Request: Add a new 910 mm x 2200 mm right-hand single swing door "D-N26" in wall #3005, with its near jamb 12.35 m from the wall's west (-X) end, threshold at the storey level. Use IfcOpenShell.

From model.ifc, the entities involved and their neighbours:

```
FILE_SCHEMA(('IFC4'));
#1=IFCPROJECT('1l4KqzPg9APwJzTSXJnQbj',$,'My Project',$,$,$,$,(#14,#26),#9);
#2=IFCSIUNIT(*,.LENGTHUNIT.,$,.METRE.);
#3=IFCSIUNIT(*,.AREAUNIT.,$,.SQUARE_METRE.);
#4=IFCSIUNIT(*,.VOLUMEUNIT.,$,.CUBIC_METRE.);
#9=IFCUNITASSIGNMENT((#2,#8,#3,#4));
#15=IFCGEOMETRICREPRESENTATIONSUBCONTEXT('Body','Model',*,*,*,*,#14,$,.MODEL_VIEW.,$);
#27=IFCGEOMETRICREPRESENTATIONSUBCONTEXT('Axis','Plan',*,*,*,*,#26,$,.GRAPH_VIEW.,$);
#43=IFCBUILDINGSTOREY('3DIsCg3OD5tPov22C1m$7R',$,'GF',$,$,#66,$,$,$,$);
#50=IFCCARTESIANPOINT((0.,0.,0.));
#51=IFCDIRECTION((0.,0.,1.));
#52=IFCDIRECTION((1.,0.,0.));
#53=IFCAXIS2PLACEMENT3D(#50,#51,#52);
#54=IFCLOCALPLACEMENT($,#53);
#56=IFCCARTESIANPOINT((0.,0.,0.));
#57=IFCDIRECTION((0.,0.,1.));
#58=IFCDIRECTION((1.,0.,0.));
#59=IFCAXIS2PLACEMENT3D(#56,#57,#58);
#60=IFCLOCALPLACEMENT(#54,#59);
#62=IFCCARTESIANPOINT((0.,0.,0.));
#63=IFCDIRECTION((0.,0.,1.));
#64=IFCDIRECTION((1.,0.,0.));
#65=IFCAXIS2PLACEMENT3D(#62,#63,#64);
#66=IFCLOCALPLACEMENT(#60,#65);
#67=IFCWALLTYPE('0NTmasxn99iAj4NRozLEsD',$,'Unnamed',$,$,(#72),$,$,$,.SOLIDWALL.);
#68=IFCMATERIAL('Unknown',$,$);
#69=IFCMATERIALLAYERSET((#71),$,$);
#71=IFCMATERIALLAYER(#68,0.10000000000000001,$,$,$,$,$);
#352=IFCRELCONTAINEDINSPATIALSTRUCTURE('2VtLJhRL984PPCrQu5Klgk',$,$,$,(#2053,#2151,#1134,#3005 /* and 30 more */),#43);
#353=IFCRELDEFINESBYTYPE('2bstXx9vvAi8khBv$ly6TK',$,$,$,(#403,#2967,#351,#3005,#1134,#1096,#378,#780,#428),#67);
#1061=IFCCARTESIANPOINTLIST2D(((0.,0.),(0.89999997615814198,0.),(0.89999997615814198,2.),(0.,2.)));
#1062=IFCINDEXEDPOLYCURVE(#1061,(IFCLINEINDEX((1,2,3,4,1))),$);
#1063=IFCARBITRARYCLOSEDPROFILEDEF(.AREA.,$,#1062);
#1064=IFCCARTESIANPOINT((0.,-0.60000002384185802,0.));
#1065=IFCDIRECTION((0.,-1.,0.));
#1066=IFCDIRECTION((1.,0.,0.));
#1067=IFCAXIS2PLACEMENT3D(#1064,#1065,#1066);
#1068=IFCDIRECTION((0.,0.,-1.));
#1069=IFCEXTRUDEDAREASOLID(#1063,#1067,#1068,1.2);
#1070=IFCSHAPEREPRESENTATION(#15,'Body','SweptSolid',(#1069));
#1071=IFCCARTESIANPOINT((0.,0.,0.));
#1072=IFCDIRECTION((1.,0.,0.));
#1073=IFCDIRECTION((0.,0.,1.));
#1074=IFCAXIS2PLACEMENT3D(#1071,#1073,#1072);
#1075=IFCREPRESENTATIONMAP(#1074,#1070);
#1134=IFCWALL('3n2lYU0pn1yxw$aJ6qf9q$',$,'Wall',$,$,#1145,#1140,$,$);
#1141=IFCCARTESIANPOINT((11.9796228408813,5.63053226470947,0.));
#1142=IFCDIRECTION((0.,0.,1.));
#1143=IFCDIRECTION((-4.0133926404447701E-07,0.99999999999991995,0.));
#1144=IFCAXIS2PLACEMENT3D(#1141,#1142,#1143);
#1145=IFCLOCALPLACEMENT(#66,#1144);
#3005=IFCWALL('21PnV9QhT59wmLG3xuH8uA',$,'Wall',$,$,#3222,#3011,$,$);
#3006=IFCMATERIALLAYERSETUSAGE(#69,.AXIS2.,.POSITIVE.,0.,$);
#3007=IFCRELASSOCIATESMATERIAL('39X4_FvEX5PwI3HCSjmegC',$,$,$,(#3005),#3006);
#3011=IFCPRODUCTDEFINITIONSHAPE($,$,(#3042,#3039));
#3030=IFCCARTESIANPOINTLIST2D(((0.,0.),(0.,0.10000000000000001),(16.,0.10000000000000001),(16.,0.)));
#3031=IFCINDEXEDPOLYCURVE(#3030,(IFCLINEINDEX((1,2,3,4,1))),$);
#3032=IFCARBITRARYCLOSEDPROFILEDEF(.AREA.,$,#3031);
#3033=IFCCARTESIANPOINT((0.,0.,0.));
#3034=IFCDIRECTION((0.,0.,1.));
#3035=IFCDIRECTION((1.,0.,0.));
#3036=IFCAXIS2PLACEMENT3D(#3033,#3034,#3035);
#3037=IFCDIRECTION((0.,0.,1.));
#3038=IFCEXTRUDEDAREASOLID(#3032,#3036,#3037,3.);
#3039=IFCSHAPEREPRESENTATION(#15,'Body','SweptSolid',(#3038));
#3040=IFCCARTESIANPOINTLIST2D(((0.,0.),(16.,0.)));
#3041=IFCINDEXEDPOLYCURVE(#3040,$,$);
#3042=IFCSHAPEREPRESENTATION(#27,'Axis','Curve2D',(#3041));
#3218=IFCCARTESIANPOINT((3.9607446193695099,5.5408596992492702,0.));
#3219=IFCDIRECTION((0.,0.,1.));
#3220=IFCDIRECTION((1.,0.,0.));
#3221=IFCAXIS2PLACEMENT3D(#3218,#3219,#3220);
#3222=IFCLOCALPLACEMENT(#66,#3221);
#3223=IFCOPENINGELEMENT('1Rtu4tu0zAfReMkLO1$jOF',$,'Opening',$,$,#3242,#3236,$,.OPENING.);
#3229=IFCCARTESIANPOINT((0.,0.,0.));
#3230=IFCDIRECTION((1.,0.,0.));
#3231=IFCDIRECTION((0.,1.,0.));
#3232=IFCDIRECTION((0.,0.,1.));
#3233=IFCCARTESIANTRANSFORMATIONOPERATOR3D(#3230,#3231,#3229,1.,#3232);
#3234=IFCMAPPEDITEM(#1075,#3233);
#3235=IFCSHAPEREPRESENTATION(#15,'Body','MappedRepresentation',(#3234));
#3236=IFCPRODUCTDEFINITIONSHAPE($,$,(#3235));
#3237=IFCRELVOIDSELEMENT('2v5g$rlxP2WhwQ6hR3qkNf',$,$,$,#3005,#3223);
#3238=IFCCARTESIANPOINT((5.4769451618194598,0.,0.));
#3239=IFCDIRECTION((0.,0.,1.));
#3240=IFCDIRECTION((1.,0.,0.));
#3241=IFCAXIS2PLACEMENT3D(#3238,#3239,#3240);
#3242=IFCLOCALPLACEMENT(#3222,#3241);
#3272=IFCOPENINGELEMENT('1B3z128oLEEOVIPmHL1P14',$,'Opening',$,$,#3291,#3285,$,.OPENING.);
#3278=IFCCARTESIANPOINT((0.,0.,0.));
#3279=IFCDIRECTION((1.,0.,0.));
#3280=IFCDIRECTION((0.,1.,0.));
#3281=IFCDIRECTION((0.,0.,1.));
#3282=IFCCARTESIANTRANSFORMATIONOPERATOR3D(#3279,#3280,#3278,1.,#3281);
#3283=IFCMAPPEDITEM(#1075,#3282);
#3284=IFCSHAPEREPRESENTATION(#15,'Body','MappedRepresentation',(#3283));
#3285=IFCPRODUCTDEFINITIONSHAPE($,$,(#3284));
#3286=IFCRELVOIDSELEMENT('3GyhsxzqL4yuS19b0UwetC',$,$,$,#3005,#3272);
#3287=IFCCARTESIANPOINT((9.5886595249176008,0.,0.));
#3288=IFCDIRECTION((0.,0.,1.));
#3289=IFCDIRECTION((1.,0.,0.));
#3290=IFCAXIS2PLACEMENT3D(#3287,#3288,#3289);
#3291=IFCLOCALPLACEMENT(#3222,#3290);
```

```python
import numpy as np
import ifcopenshell
import ifcopenshell.api.feature
import ifcopenshell.api.geometry
import ifcopenshell.api.root
import ifcopenshell.api.spatial
import ifcopenshell.geom
import ifcopenshell.util.element
import ifcopenshell.util.placement
import ifcopenshell.util.representation
import ifcopenshell.util.shape
import ifcopenshell.util.unit

model = ifcopenshell.open("model.ifc")
unit_scale = ifcopenshell.util.unit.calculate_unit_scale(model)
settings = ifcopenshell.geom.settings()


def volume(element):
    """Net volume in cubic metres, openings subtracted."""
    shape = ifcopenshell.geom.create_shape(settings, element)
    return ifcopenshell.util.shape.get_volume(shape.geometry)


wall = model.by_id(3005)
storey = ifcopenshell.util.element.get_container(wall, ifc_class="IfcBuildingStorey")
context = ifcopenshell.util.representation.get_context(model, "Model", "Body", "MODEL_VIEW")
before = volume(wall)

width, height, from_end, sill = 0.91, 2.2, 12.35, 0.0  # metres

# The wall runs along its own X axis, and the end named is its -X end.
wall_shape = ifcopenshell.geom.create_shape(settings, wall)
x, y, z = ifcopenshell.util.shape.get_vertices(wall_shape.geometry).T
start = x.min() + from_end
face, thickness = float(y.min()), float(y.max() - y.min())
wall_matrix = ifcopenshell.util.placement.get_local_placement(wall.ObjectPlacement)
level = ifcopenshell.util.placement.get_local_placement(storey.ObjectPlacement)[2, 3]


def in_wall(x, y):
    """Placement at x, y metres in the wall's axes, at sill height."""
    matrix = wall_matrix.copy()
    matrix[:, 3] = wall_matrix @ np.array([x / unit_scale, y / unit_scale, 0.0, 1.0])
    matrix[2, 3] = level + sill / unit_scale
    return matrix


# Opening: a box that overshoots both wall faces by 50 mm.
opening = ifcopenshell.api.root.create_entity(model, ifc_class="IfcOpeningElement", predefined_type="OPENING")
box = ifcopenshell.api.geometry.add_wall_representation(
    model, context=context, length=width, height=height, thickness=thickness + 0.1
)
ifcopenshell.api.geometry.assign_representation(model, product=opening, representation=box)
ifcopenshell.api.geometry.edit_object_placement(model, product=opening, matrix=in_wall(start, face - 0.05), is_si=False)
ifcopenshell.api.feature.add_feature(model, feature=opening, element=wall)

door = ifcopenshell.api.root.create_entity(model, ifc_class="IfcDoor", name="D-N26", predefined_type="DOOR")
door.OverallWidth, door.OverallHeight = width / unit_scale, height / unit_scale
door.OperationType = "SINGLE_SWING_RIGHT"
body = ifcopenshell.api.geometry.add_door_representation(
    model,
    context=context,
    overall_width=door.OverallWidth,
    overall_height=door.OverallHeight,
    operation_type="SINGLE_SWING_RIGHT",
    lining_properties={"LiningDepth": thickness / unit_scale, "ThresholdDepth": thickness / unit_scale},
)
ifcopenshell.api.geometry.assign_representation(model, product=door, representation=body)
ifcopenshell.api.spatial.assign_container(model, products=[door], relating_structure=storey)
ifcopenshell.api.feature.add_filling(model, opening=opening, element=door)

# The lining spans the wall, so the door starts at the wall face.
ifcopenshell.api.geometry.edit_object_placement(model, product=door, matrix=in_wall(start, face), is_si=False)

after = volume(wall)

print(f"wall volume {before:.3f} -> {after:.3f} m3")

model.write("model_rev.ifc")
```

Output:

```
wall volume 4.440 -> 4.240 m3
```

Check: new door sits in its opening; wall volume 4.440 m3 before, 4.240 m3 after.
